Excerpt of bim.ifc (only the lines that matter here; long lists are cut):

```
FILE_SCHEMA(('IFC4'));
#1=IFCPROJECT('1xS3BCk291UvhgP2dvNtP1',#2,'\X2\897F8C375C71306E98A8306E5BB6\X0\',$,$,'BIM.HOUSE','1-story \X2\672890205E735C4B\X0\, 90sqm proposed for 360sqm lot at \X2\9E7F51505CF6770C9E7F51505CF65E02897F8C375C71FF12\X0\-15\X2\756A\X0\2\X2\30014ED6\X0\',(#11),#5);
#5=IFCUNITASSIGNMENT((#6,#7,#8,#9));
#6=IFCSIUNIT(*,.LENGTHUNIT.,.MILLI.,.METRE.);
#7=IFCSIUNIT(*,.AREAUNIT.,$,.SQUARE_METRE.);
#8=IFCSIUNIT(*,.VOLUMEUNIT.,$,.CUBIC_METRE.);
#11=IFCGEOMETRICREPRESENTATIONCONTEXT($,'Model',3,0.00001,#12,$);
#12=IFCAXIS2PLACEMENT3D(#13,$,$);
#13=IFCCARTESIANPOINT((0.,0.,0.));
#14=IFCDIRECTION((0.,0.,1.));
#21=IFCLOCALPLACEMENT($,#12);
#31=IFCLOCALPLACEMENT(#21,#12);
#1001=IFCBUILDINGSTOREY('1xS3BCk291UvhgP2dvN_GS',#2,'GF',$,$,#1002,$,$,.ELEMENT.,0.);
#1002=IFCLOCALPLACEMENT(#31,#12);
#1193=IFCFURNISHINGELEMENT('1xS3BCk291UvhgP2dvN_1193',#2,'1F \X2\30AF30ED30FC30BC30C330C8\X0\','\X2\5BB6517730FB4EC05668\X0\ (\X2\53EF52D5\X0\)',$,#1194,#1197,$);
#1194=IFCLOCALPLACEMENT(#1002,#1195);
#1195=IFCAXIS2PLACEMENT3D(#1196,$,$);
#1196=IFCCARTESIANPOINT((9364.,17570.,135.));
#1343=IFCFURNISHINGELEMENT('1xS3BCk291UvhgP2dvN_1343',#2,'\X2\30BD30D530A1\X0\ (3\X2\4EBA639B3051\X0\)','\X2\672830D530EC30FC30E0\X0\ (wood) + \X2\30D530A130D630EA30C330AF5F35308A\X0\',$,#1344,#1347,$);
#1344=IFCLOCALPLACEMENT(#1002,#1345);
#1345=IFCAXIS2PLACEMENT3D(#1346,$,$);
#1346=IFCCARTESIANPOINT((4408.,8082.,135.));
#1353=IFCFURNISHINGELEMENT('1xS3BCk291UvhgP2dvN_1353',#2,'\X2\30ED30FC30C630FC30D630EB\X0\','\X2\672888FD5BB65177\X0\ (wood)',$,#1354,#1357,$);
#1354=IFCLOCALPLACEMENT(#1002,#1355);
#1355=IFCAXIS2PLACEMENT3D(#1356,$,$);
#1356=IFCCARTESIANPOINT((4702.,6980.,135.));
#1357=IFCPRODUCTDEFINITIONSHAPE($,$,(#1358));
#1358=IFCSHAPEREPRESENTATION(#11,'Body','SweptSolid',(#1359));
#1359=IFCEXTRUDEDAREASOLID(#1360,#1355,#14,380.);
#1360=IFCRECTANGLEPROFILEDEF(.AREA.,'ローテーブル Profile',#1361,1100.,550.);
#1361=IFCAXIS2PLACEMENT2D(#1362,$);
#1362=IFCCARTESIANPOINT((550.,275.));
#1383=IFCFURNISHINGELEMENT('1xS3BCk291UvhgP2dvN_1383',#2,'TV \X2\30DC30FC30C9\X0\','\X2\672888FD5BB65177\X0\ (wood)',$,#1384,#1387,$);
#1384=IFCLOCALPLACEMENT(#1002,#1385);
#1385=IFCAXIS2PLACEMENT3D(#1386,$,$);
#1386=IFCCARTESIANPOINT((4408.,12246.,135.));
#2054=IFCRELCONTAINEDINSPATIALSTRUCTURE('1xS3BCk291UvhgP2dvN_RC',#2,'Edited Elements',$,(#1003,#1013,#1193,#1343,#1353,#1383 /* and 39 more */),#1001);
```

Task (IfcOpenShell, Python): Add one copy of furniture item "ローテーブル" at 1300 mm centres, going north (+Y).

```python
import numpy as np
import ifcopenshell
import ifcopenshell.api.geometry
import ifcopenshell.api.root
import ifcopenshell.util.element
import ifcopenshell.util.placement

model = ifcopenshell.open("bim.ifc")


def reuse_history(source, copy):
    """copy_class also copies each property set's owner history, people and application; keep the originals."""
    for rel in copy.IsDefinedBy:
        if rel.is_a("IfcRelDefinesByProperties") and (history := rel.RelatingPropertyDefinition.OwnerHistory):
            rel.RelatingPropertyDefinition.OwnerHistory = source.OwnerHistory
            ifcopenshell.util.element.remove_deep2(model, history)


source = model.by_id(1353)
base = ifcopenshell.util.placement.get_local_placement(source.ObjectPlacement)
step = np.array([0.0, 1.0, 0.0]) * 1300.0

for i in range(1, 2):
    copy = ifcopenshell.api.root.copy_class(model, product=source)
    copy.Representation = ifcopenshell.util.element.copy_deep(
        model, source.Representation, exclude=["IfcGeometricRepresentationContext", "IfcRepresentationMap"]
    )
    reuse_history(source, copy)
    matrix = base.copy()
    matrix[:3, 3] += i * step
    print("added at", matrix[:3, 3].round(3) + 0.0)
    ifcopenshell.api.geometry.edit_object_placement(model, product=copy, matrix=matrix, is_si=False)

model.write("bim-out.ifc")
```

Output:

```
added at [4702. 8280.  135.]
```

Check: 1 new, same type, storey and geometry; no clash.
